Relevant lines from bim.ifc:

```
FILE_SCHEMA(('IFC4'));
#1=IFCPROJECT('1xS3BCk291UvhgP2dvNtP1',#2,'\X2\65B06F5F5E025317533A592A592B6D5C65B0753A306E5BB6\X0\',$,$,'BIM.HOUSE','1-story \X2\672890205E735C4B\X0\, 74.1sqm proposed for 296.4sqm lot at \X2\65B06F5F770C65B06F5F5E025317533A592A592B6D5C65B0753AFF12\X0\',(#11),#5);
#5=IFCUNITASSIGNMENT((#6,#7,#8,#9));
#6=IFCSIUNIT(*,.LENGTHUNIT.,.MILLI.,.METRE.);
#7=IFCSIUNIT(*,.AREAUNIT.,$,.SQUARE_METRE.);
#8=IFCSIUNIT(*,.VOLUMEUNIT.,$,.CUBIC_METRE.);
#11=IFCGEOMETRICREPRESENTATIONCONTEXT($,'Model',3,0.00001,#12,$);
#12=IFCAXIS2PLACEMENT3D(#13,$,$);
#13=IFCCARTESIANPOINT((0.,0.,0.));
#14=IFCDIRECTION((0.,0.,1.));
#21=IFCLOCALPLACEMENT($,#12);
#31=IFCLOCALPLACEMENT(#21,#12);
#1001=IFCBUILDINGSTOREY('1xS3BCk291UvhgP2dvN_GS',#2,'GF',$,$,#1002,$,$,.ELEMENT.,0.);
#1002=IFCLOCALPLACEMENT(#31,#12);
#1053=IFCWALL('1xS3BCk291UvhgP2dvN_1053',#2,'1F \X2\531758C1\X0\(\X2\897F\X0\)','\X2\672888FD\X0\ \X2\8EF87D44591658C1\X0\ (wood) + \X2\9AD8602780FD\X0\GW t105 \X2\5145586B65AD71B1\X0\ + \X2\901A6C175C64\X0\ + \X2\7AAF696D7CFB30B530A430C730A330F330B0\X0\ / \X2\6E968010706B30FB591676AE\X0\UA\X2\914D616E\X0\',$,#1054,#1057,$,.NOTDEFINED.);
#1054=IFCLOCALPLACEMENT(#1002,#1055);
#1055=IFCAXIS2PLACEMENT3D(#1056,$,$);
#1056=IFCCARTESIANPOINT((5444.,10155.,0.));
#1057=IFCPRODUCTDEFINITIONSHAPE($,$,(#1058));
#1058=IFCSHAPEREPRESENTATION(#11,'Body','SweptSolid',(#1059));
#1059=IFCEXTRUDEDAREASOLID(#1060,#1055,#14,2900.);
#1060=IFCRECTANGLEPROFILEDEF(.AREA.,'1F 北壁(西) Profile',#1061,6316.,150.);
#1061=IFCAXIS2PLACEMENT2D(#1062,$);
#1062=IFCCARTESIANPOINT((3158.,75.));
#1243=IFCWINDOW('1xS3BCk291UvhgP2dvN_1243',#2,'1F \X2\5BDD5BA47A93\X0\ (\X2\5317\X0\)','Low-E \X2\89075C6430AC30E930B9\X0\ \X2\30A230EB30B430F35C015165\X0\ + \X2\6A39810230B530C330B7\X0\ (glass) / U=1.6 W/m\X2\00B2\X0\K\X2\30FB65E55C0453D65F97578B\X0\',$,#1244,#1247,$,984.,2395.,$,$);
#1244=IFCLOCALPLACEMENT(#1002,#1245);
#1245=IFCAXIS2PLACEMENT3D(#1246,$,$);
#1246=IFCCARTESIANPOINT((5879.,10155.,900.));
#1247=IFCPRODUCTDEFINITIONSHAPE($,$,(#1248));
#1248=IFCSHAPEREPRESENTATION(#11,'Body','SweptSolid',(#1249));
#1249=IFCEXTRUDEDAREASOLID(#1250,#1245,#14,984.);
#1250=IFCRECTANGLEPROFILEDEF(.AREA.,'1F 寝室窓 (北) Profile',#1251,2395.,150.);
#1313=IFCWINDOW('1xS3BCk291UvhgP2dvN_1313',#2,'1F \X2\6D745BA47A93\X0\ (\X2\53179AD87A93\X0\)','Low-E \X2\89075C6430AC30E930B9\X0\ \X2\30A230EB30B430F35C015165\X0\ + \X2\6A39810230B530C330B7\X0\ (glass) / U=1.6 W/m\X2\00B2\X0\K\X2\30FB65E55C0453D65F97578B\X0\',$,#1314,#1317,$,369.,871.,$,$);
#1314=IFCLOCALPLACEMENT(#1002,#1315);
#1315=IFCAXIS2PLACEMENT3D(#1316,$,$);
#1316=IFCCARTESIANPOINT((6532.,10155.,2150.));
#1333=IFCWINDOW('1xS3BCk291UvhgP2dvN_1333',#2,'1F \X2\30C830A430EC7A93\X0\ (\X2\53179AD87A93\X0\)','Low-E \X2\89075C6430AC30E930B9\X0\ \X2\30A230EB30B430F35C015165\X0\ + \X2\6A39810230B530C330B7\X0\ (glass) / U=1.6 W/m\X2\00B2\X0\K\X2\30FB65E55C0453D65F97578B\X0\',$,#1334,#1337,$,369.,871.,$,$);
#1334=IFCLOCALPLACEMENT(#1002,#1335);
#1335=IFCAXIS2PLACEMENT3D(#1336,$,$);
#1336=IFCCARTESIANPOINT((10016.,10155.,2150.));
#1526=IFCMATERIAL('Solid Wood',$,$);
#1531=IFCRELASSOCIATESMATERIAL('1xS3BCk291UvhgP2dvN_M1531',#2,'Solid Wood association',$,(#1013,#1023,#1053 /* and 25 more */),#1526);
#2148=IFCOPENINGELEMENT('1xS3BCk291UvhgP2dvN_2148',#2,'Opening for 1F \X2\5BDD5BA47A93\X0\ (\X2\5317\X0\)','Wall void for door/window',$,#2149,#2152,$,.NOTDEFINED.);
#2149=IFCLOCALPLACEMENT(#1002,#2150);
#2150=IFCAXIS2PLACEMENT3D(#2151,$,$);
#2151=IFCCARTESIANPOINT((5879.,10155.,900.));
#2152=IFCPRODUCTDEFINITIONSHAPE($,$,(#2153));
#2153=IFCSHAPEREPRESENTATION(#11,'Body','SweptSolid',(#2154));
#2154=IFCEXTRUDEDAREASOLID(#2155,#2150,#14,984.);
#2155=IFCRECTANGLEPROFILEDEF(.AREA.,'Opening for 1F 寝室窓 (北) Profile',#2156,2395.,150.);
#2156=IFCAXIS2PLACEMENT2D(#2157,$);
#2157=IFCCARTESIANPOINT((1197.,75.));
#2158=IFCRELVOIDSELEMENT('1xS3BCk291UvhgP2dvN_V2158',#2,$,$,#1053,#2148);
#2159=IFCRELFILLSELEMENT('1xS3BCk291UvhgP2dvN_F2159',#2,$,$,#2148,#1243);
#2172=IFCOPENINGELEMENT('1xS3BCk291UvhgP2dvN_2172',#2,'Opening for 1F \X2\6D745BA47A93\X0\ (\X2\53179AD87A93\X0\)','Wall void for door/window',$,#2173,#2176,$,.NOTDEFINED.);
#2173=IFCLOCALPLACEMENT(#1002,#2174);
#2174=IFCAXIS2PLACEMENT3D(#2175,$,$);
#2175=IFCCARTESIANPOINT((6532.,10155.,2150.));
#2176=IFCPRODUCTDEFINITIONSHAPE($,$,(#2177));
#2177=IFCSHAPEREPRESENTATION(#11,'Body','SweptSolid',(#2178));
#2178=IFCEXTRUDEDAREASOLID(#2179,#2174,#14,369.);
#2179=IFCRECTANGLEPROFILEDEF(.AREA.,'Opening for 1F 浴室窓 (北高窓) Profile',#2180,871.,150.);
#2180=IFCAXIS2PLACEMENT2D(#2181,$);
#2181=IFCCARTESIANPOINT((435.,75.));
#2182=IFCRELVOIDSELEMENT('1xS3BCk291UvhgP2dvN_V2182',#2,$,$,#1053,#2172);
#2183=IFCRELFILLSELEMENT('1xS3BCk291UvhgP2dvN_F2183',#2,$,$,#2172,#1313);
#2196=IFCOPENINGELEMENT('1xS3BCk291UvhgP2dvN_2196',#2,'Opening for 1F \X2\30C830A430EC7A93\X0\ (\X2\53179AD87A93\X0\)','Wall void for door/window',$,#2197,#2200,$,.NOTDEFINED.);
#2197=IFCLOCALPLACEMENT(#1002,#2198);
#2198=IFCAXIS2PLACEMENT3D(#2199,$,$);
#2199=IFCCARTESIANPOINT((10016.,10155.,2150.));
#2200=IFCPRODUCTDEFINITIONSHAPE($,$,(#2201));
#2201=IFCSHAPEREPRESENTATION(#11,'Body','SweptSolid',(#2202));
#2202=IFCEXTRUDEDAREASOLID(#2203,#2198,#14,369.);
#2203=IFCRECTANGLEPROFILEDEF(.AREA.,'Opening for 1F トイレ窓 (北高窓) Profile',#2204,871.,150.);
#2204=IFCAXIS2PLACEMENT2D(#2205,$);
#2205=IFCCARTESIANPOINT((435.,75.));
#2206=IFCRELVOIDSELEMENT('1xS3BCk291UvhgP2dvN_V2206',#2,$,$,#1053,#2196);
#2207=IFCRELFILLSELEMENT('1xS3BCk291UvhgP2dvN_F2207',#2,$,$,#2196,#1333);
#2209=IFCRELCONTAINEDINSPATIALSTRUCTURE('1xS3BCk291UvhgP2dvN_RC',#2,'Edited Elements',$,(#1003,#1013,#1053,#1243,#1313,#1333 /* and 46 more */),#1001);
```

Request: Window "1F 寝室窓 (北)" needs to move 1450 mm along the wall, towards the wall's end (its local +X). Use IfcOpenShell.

```python
import ifcopenshell
import ifcopenshell.api.geometry
import ifcopenshell.util.placement
import ifcopenshell.util.unit

model = ifcopenshell.open("bim.ifc")
unit_scale = ifcopenshell.util.unit.calculate_unit_scale(model)

window = model.by_guid("1xS3BCk291UvhgP2dvN_1243")
opening = window.FillsVoids[0].RelatingOpeningElement
wall = opening.VoidsElements[0].RelatingBuildingElement

wall_matrix = ifcopenshell.util.placement.get_local_placement(wall.ObjectPlacement)
shift = wall_matrix[:3, 0] * 1.45 / unit_scale
before = ifcopenshell.util.placement.get_local_placement(window.ObjectPlacement)[:3, 3].copy()

# The window is not placed relative to its opening, so move both.
for product in (opening, window):
    matrix = ifcopenshell.util.placement.get_local_placement(product.ObjectPlacement)
    matrix[:3, 3] += shift
    ifcopenshell.api.geometry.edit_object_placement(model, product=product, matrix=matrix, is_si=False)

after = ifcopenshell.util.placement.get_local_placement(window.ObjectPlacement)[:3, 3]
print("window moved by", (after - before).round(3) + 0.0)

model.write("bim_edited.ifc")
```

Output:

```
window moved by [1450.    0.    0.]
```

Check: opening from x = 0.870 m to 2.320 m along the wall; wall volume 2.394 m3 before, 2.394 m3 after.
